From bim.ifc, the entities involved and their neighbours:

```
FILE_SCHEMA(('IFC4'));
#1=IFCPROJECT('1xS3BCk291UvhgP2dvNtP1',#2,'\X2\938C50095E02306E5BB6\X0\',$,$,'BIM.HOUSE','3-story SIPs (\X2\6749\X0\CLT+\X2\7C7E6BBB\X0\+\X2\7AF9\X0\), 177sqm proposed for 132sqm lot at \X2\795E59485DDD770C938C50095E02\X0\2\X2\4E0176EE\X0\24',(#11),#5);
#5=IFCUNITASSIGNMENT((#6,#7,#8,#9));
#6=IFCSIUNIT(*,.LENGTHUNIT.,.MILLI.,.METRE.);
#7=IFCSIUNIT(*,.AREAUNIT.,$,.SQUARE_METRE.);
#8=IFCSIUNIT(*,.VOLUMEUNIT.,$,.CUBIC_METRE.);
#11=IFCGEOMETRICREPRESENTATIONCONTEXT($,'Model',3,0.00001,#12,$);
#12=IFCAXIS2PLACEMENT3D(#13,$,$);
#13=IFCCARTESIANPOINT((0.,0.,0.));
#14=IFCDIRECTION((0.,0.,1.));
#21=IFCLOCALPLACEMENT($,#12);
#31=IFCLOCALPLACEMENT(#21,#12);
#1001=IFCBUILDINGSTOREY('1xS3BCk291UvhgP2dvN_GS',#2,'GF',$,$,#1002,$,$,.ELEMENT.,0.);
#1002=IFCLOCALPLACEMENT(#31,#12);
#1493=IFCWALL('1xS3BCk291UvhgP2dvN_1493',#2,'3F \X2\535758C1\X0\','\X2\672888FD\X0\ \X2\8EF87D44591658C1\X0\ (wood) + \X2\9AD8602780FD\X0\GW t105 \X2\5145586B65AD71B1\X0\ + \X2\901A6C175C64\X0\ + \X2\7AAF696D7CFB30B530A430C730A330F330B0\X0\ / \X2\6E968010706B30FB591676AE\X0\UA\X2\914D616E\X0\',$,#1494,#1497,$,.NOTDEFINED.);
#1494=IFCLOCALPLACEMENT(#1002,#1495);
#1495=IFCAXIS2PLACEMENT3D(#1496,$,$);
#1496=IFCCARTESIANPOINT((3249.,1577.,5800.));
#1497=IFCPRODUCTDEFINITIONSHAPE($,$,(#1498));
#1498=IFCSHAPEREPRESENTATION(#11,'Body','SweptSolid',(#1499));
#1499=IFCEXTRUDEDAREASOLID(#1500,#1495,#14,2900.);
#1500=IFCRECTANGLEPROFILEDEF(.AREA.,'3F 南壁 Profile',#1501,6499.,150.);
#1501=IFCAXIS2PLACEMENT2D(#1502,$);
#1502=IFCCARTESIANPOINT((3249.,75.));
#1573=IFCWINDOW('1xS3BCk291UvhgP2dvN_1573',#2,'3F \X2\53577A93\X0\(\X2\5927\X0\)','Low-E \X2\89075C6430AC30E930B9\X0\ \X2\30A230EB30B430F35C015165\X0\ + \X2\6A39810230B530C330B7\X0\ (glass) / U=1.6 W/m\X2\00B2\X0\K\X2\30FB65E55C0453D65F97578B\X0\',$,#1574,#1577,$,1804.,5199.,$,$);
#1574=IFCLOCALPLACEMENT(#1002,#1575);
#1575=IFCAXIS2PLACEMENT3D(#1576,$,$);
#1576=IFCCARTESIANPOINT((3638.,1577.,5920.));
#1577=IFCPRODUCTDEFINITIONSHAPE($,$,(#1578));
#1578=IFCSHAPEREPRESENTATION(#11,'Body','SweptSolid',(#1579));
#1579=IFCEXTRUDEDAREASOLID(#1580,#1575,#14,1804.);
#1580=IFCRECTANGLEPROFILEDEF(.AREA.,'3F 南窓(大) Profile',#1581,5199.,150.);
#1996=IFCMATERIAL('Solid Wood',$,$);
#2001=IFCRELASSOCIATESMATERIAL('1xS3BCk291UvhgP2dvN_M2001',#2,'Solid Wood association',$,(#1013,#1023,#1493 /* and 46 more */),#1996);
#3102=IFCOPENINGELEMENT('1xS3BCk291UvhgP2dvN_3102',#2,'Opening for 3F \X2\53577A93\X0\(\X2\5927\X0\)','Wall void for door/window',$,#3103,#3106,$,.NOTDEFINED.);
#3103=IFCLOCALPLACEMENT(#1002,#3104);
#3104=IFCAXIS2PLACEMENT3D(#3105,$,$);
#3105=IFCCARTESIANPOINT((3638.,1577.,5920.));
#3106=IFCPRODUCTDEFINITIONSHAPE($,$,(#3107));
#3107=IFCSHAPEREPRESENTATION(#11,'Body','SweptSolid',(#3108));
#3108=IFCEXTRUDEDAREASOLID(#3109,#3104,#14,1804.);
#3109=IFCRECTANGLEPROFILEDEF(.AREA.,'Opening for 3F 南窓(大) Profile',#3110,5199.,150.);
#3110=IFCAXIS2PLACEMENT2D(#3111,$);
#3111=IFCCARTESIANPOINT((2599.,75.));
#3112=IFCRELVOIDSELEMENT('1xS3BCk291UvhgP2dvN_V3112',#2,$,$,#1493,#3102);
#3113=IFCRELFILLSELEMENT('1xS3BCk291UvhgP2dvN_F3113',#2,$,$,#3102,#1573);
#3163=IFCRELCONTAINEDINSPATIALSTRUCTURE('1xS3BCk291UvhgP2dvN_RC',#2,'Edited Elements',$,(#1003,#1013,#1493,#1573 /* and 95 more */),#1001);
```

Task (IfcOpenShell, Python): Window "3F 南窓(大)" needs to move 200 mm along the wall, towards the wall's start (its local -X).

```python
import ifcopenshell
import ifcopenshell.api.geometry
import ifcopenshell.util.placement
import ifcopenshell.util.unit

model = ifcopenshell.open("bim.ifc")
unit_scale = ifcopenshell.util.unit.calculate_unit_scale(model)

window = model.by_id(1573)
opening = window.FillsVoids[0].RelatingOpeningElement
wall = opening.VoidsElements[0].RelatingBuildingElement

wall_matrix = ifcopenshell.util.placement.get_local_placement(wall.ObjectPlacement)
shift = wall_matrix[:3, 0] * -0.2 / unit_scale
before = ifcopenshell.util.placement.get_local_placement(window.ObjectPlacement)[:3, 3].copy()

# The window is not placed relative to its opening, so move both.
for product in (opening, window):
    matrix = ifcopenshell.util.placement.get_local_placement(product.ObjectPlacement)
    matrix[:3, 3] += shift
    ifcopenshell.api.geometry.edit_object_placement(model, product=product, matrix=matrix, is_si=False)

after = ifcopenshell.util.placement.get_local_placement(window.ObjectPlacement)[:3, 3]
print("window moved by", (after - before).round(3) + 0.0)

model.write("bim_edited.ifc")
```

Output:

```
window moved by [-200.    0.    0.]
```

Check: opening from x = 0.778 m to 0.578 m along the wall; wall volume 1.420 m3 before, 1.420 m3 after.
